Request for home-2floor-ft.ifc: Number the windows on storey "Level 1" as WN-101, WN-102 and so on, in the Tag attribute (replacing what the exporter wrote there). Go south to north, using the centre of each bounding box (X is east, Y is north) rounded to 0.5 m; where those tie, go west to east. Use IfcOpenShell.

First a look at what the model holds.

```python
import ifcopenshell
import ifcopenshell.util.element
import ifcopenshell.util.placement

model = ifcopenshell.open("home-2floor-ft.ifc")
print(model.schema)
storey = next(s for s in model.by_type("IfcBuildingStorey") if s.Name == "Level 1")
windows = [e for e in ifcopenshell.util.element.get_decomposition(storey) if e.is_a("IfcWindow")]
for e in sorted(windows, key=lambda e: e.id()):
    origin = ifcopenshell.util.placement.get_local_placement(e.ObjectPlacement)[:3, 3]
    print(e.id(), e.Tag, e.Name, origin.round(2) + 0.0, sep=" | ")
```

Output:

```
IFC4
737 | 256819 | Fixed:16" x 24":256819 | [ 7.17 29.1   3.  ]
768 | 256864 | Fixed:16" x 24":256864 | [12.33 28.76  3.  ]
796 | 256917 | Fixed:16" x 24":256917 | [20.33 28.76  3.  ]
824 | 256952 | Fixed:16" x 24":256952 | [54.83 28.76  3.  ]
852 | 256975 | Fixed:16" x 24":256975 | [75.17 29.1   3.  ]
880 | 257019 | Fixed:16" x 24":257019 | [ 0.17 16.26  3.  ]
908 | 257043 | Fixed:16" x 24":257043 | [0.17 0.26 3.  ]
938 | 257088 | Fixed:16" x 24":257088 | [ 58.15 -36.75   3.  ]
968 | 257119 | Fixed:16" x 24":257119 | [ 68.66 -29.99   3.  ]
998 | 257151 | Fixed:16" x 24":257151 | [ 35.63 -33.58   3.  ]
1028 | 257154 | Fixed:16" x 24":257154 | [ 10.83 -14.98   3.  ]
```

```python
import ifcopenshell
import ifcopenshell.geom
import ifcopenshell.util.element
import ifcopenshell.util.shape

model = ifcopenshell.open("home-2floor-ft.ifc")
settings = ifcopenshell.geom.settings()
settings.set("use-world-coords", True)


def centre(element):
    shape = ifcopenshell.geom.create_shape(settings, element)
    return ifcopenshell.util.shape.get_bbox_centroid(shape.geometry)


storey = next(s for s in model.by_type("IfcBuildingStorey") if s.Name == "Level 1")
windows = [e for e in ifcopenshell.util.element.get_decomposition(storey) if e.is_a("IfcWindow")]

# Insertion points can sit at a corner or the storey origin, so sort by the geometry (in metres).
centres = {e: centre(e) for e in windows}
windows.sort(key=lambda e: (round(centres[e][1] / 0.5), centres[e][0]))

for i, e in enumerate(windows, start=1):
    number = f"WN-1{i:02d}"
    e.Tag = number
    print(e.id(), number)

model.write("home-2floor-ft-out.ifc")
```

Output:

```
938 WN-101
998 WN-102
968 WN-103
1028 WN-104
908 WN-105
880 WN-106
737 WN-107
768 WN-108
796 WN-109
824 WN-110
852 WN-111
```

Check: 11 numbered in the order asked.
